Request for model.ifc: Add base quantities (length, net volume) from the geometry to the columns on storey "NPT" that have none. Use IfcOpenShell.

First a look at what the model holds.

```python
import ifcopenshell
import ifcopenshell.util.element
import ifcopenshell.util.unit

model = ifcopenshell.open("model.ifc")
print(model.schema)
for unit_type in ("LENGTHUNIT", "AREAUNIT", "VOLUMEUNIT"):
    print(unit_type, ifcopenshell.util.unit.calculate_unit_scale(model, unit_type))
storey = next(s for s in model.by_type("IfcBuildingStorey") if s.Name == "NPT")
columns = [e for e in ifcopenshell.util.element.get_decomposition(storey) if e.is_a("IfcColumn")]
for e in sorted(columns, key=lambda e: e.id()):
    print(e.id(), e.is_a(), e.Name, list(ifcopenshell.util.element.get_psets(e, qtos_only=True)), sep=" | ")
```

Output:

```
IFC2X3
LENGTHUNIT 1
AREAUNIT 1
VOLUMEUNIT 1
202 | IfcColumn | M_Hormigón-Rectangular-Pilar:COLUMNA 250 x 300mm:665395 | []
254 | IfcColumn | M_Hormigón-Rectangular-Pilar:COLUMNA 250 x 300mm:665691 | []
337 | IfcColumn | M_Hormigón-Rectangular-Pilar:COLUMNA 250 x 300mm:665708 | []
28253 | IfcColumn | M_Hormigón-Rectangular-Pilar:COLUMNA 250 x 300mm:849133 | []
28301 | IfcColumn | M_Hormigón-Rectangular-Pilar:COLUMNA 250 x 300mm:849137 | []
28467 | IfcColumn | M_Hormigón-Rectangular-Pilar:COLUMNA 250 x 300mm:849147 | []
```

```python
import ifcopenshell
import ifcopenshell.api.pset
import ifcopenshell.geom
import ifcopenshell.util.element
import ifcopenshell.util.shape
import ifcopenshell.util.unit

model = ifcopenshell.open("model.ifc")
unit_scale = ifcopenshell.util.unit.calculate_unit_scale(model)
volume_scale = ifcopenshell.util.unit.calculate_unit_scale(model, "VOLUMEUNIT")
settings = ifcopenshell.geom.settings()

storey = next(s for s in model.by_type("IfcBuildingStorey") if s.Name == "NPT")
columns = [e for e in ifcopenshell.util.element.get_decomposition(storey) if e.is_a("IfcColumn")]

for e in sorted(columns, key=lambda e: e.id()):
    if ifcopenshell.util.element.get_psets(e, qtos_only=True, should_inherit=False):
        continue
    # Geometry comes back in metres, in the element's own axes.
    shape = ifcopenshell.geom.create_shape(settings, e)
    values = {
        "Length": ifcopenshell.util.shape.get_z(shape.geometry) / unit_scale,
        "NetVolume": ifcopenshell.util.shape.get_volume(shape.geometry) / volume_scale,
    }
    qto = ifcopenshell.api.pset.add_qto(model, product=e, name="BaseQuantities")
    ifcopenshell.api.pset.edit_qto(model, qto=qto, properties=values)
    print(e.id(), {k: round(v, 3) for k, v in values.items()})

model.write("model-out.ifc")
```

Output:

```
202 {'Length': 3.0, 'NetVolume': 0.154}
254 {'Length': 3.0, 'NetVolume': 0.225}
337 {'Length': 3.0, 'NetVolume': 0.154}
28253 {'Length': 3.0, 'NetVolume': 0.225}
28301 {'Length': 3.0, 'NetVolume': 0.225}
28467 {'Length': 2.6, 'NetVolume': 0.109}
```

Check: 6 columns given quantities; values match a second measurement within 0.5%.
